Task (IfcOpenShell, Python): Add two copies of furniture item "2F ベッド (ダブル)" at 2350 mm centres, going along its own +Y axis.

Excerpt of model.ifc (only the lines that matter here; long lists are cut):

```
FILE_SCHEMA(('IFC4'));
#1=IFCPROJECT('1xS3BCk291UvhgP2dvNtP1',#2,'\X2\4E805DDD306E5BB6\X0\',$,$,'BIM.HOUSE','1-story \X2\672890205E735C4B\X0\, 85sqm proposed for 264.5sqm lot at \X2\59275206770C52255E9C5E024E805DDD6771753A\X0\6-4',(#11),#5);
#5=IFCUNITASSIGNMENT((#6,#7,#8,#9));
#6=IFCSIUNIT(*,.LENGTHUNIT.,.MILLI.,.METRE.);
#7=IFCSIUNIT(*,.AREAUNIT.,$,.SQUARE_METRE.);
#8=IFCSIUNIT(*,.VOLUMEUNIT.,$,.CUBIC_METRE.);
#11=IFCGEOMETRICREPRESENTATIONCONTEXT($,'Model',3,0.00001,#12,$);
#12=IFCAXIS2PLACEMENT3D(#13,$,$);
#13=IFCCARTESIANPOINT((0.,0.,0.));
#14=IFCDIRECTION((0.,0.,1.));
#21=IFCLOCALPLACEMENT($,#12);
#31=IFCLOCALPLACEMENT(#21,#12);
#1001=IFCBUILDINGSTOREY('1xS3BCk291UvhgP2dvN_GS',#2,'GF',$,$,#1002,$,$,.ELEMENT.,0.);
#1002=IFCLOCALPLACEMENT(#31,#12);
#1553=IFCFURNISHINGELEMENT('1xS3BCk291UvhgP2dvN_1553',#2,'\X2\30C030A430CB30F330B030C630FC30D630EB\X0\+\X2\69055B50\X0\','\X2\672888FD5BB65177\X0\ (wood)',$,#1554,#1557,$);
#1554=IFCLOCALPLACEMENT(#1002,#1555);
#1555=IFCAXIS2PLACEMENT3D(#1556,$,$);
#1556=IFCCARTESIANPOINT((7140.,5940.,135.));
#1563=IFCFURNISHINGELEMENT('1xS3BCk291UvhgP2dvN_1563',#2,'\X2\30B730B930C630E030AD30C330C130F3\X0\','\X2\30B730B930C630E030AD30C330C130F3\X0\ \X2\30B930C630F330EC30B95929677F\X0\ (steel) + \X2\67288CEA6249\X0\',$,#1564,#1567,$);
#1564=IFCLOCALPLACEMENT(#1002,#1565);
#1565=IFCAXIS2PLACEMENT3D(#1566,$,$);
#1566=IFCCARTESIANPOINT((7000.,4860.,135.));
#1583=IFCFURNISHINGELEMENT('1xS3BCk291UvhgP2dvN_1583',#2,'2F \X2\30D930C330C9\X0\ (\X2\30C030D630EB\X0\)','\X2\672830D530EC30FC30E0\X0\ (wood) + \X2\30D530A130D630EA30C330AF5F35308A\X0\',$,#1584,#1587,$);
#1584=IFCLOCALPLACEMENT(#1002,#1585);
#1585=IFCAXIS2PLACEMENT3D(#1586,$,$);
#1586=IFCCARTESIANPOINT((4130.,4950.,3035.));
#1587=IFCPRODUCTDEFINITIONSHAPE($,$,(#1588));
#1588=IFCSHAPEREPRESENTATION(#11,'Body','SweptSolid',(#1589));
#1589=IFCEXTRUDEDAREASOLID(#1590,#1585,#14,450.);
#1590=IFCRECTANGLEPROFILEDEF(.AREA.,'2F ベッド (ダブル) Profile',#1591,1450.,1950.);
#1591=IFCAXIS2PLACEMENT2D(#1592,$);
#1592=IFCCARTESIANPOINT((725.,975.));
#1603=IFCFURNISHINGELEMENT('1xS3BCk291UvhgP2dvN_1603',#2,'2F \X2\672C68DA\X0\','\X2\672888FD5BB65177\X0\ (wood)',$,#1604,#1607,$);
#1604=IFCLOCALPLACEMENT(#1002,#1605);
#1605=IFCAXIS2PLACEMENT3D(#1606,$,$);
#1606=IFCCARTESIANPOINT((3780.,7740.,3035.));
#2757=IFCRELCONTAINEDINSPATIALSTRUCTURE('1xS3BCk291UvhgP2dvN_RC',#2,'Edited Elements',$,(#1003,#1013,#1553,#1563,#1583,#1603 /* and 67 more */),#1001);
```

```python
import ifcopenshell
import ifcopenshell.api.geometry
import ifcopenshell.api.root
import ifcopenshell.util.element
import ifcopenshell.util.placement
import ifcopenshell.util.unit

model = ifcopenshell.open("model.ifc")
unit_scale = ifcopenshell.util.unit.calculate_unit_scale(model)


def reuse_history(source, copy):
    """copy_class also copies each property set's owner history, people and application; keep the originals."""
    for rel in copy.IsDefinedBy:
        if rel.is_a("IfcRelDefinesByProperties") and (history := rel.RelatingPropertyDefinition.OwnerHistory):
            rel.RelatingPropertyDefinition.OwnerHistory = source.OwnerHistory
            ifcopenshell.util.element.remove_deep2(model, history)


source = model.by_guid("1xS3BCk291UvhgP2dvN_1583")
base = ifcopenshell.util.placement.get_local_placement(source.ObjectPlacement)
step = base[:3, 1] * 2.35 / unit_scale

for i in range(1, 3):
    copy = ifcopenshell.api.root.copy_class(model, product=source)
    copy.Representation = ifcopenshell.util.element.copy_deep(
        model, source.Representation, exclude=["IfcGeometricRepresentationContext", "IfcRepresentationMap"]
    )
    reuse_history(source, copy)
    matrix = base.copy()
    matrix[:3, 3] += i * step
    print("added at", matrix[:3, 3].round(3) + 0.0)
    ifcopenshell.api.geometry.edit_object_placement(model, product=copy, matrix=matrix, is_si=False)

model.write("model_edited.ifc")
```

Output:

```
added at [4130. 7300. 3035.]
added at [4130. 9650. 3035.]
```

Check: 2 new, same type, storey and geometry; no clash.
